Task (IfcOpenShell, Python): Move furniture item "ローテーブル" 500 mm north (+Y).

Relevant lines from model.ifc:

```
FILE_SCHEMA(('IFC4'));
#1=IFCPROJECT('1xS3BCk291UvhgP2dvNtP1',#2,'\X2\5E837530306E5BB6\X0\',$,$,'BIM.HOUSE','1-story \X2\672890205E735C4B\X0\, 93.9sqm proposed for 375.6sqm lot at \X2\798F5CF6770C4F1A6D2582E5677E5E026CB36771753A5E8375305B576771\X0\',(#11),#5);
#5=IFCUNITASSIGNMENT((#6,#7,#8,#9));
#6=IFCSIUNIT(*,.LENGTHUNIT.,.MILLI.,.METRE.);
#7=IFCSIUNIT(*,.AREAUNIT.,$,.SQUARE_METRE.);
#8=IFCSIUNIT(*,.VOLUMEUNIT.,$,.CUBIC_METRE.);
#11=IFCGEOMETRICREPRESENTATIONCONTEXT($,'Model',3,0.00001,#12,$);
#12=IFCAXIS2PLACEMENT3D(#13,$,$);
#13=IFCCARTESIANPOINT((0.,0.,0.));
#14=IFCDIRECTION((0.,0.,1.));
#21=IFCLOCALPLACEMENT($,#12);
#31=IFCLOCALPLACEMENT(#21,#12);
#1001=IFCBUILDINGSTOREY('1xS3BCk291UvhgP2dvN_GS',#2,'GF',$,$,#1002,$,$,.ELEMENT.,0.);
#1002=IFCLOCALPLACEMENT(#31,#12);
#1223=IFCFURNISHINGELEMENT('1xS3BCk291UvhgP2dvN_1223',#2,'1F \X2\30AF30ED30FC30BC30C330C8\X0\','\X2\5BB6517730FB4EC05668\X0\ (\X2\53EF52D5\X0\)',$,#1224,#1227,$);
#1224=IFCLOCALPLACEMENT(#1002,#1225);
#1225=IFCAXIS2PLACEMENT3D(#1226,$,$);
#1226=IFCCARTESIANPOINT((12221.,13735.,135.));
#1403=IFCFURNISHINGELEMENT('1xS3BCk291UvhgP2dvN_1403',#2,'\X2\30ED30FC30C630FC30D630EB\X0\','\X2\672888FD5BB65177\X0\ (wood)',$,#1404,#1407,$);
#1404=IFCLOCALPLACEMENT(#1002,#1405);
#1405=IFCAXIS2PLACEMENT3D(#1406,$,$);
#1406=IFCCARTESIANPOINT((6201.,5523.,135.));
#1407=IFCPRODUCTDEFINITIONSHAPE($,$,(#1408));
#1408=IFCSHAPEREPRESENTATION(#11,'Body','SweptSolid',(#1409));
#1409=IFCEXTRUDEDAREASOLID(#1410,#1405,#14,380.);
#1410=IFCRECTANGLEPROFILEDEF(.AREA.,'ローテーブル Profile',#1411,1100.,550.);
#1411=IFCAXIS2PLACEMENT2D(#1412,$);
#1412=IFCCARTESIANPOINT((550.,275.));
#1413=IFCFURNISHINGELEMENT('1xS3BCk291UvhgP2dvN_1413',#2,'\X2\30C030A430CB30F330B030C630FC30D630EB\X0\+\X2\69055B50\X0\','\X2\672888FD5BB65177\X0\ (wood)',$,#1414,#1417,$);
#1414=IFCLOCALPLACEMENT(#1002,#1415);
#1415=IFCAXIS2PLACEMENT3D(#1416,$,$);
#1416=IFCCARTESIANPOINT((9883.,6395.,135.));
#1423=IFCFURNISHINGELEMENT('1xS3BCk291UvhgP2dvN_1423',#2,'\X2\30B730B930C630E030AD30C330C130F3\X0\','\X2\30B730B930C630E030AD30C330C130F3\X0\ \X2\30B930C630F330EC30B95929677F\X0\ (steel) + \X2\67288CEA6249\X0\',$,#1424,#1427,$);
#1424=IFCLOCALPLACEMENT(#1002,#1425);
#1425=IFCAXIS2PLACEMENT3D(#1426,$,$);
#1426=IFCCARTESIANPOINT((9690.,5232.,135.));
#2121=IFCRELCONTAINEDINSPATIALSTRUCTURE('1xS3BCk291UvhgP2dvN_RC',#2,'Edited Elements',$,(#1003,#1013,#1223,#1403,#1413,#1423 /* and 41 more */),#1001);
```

```python
import ifcopenshell
import ifcopenshell.api.geometry
import ifcopenshell.util.placement
import ifcopenshell.util.unit

model = ifcopenshell.open("model.ifc")
unit_scale = ifcopenshell.util.unit.calculate_unit_scale(model)

item = model.by_guid("1xS3BCk291UvhgP2dvN_1403")
matrix = ifcopenshell.util.placement.get_local_placement(item.ObjectPlacement)
matrix[1, 3] += 0.5 / unit_scale
ifcopenshell.api.geometry.edit_object_placement(model, product=item, matrix=matrix, is_si=False)

print(ifcopenshell.util.placement.get_local_placement(item.ObjectPlacement).round(3) + 0.0)

model.write("model-out.ifc")
```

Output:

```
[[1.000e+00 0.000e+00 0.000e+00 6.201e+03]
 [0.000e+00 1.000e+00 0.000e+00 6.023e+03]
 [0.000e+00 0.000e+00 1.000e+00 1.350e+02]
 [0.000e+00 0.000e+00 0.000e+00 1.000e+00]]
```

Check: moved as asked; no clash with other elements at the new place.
